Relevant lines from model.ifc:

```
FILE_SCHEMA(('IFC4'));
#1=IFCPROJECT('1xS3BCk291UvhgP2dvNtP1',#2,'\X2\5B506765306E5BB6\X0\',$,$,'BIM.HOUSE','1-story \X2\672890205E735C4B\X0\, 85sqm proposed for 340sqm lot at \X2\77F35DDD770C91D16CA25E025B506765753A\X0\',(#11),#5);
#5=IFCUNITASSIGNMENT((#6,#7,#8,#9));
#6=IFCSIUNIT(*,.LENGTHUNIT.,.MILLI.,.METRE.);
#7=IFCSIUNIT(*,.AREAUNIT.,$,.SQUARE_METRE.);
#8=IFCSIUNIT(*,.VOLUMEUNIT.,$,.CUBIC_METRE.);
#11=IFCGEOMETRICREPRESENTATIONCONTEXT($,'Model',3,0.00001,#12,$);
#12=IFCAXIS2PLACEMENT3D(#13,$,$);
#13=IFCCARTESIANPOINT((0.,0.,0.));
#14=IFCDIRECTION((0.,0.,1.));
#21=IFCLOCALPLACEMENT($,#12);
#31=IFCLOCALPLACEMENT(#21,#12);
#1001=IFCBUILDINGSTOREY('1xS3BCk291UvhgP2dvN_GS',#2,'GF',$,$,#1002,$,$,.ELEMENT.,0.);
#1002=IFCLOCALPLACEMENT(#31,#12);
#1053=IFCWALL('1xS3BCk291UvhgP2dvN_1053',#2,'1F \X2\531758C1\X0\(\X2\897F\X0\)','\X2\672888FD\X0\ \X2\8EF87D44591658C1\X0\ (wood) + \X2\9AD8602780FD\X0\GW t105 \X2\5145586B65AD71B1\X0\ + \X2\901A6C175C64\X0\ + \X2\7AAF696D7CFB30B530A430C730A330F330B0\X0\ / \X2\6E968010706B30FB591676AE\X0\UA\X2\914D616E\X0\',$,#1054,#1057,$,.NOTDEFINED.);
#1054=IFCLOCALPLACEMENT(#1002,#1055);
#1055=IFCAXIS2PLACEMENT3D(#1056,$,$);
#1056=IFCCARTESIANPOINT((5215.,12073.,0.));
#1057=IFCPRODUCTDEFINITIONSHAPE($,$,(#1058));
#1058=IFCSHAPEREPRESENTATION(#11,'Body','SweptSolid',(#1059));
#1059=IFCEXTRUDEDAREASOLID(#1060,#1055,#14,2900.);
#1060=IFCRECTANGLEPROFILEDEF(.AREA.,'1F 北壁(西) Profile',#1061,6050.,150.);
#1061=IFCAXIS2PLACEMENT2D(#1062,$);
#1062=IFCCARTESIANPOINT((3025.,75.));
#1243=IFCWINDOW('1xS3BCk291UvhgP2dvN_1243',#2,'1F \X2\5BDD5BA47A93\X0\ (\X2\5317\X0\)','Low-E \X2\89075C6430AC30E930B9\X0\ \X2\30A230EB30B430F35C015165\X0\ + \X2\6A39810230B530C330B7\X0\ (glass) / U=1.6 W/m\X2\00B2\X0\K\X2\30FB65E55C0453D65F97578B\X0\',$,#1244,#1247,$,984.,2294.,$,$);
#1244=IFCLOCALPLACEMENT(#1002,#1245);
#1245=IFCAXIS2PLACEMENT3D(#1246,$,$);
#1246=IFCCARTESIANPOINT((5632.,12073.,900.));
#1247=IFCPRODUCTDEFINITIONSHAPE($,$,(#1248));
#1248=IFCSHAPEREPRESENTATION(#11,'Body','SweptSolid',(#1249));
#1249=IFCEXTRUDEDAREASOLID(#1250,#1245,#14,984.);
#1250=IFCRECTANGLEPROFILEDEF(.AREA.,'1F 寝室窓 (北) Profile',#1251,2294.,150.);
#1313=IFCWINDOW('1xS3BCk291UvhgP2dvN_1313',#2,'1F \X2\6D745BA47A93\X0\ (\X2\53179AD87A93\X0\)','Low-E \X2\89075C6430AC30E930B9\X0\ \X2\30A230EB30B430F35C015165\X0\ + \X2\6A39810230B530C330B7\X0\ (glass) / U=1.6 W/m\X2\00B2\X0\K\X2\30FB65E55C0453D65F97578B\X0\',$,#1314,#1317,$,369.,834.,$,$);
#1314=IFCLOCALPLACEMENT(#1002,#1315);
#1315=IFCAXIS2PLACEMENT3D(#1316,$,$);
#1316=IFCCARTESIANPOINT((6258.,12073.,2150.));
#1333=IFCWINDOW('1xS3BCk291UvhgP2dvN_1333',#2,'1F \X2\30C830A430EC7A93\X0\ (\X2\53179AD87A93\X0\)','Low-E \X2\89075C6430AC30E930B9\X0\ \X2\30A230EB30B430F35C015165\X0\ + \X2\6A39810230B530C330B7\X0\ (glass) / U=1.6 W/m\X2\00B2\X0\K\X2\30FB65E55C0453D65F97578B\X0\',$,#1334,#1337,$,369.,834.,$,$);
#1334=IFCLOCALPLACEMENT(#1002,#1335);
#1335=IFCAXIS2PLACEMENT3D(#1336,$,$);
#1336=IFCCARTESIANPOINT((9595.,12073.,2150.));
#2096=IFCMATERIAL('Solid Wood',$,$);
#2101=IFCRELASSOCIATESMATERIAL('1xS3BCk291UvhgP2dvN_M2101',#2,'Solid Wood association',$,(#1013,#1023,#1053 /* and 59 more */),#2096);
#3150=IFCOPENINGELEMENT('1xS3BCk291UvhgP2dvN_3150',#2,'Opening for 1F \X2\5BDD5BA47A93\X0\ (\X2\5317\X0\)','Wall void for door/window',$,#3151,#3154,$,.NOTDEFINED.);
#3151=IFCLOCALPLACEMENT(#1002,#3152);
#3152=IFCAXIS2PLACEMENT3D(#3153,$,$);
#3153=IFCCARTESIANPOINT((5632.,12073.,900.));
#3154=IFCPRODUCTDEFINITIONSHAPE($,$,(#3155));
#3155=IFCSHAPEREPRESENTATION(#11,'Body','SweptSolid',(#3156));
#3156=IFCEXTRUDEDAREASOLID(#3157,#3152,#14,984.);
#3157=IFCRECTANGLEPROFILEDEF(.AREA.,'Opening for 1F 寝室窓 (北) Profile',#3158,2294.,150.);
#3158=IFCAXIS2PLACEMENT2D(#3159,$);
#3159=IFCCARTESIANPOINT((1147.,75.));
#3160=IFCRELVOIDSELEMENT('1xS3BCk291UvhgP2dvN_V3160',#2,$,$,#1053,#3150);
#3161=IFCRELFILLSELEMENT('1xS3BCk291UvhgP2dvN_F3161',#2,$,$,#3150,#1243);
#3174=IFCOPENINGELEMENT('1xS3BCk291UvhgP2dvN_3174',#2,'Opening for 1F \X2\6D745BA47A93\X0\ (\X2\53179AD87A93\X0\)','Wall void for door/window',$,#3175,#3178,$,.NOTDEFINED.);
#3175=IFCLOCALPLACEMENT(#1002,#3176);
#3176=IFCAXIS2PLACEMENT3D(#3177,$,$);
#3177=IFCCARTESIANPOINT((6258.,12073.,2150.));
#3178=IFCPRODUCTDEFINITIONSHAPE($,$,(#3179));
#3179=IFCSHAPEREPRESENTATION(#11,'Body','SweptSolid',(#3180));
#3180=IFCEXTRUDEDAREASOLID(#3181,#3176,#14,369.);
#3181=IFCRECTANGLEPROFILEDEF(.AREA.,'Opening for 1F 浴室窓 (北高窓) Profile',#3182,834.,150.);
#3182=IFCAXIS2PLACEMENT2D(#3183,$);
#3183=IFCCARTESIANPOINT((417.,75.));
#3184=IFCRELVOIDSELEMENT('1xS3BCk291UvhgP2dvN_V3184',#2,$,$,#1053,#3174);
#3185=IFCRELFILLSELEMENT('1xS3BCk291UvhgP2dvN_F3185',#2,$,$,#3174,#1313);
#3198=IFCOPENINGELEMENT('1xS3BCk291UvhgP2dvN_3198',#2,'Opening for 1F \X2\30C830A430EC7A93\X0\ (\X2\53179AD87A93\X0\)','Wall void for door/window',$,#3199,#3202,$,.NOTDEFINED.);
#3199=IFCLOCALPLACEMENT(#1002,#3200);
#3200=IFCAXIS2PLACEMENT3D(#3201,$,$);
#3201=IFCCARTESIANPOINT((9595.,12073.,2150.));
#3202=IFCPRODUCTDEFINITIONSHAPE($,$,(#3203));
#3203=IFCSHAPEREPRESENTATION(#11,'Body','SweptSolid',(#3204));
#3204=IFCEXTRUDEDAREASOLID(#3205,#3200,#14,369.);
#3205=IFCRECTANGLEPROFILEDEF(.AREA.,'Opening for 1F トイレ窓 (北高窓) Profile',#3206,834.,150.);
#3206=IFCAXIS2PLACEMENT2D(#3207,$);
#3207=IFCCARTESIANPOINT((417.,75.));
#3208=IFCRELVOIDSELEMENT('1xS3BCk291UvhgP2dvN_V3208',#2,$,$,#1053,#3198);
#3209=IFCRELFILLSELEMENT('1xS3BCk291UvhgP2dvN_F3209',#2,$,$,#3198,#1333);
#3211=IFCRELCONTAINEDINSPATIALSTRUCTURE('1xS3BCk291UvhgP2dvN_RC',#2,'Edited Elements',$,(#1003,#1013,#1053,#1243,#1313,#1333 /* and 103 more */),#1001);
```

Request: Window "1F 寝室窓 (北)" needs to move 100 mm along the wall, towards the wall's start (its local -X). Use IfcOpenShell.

```python
import ifcopenshell
import ifcopenshell.api.geometry
import ifcopenshell.util.placement
import ifcopenshell.util.unit

model = ifcopenshell.open("model.ifc")
unit_scale = ifcopenshell.util.unit.calculate_unit_scale(model)

window = model.by_id(1243)
opening = window.FillsVoids[0].RelatingOpeningElement
wall = opening.VoidsElements[0].RelatingBuildingElement

wall_matrix = ifcopenshell.util.placement.get_local_placement(wall.ObjectPlacement)
shift = wall_matrix[:3, 0] * -0.1 / unit_scale
before = ifcopenshell.util.placement.get_local_placement(window.ObjectPlacement)[:3, 3].copy()

# The window is not placed relative to its opening, so move both.
for product in (opening, window):
    matrix = ifcopenshell.util.placement.get_local_placement(product.ObjectPlacement)
    matrix[:3, 3] += shift
    ifcopenshell.api.geometry.edit_object_placement(model, product=product, matrix=matrix, is_si=False)

after = ifcopenshell.util.placement.get_local_placement(window.ObjectPlacement)[:3, 3]
print("window moved by", (after - before).round(3) + 0.0)

model.write("model_updated.ifc")
```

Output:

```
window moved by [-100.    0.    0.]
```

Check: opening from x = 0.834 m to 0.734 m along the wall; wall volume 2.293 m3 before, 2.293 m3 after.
